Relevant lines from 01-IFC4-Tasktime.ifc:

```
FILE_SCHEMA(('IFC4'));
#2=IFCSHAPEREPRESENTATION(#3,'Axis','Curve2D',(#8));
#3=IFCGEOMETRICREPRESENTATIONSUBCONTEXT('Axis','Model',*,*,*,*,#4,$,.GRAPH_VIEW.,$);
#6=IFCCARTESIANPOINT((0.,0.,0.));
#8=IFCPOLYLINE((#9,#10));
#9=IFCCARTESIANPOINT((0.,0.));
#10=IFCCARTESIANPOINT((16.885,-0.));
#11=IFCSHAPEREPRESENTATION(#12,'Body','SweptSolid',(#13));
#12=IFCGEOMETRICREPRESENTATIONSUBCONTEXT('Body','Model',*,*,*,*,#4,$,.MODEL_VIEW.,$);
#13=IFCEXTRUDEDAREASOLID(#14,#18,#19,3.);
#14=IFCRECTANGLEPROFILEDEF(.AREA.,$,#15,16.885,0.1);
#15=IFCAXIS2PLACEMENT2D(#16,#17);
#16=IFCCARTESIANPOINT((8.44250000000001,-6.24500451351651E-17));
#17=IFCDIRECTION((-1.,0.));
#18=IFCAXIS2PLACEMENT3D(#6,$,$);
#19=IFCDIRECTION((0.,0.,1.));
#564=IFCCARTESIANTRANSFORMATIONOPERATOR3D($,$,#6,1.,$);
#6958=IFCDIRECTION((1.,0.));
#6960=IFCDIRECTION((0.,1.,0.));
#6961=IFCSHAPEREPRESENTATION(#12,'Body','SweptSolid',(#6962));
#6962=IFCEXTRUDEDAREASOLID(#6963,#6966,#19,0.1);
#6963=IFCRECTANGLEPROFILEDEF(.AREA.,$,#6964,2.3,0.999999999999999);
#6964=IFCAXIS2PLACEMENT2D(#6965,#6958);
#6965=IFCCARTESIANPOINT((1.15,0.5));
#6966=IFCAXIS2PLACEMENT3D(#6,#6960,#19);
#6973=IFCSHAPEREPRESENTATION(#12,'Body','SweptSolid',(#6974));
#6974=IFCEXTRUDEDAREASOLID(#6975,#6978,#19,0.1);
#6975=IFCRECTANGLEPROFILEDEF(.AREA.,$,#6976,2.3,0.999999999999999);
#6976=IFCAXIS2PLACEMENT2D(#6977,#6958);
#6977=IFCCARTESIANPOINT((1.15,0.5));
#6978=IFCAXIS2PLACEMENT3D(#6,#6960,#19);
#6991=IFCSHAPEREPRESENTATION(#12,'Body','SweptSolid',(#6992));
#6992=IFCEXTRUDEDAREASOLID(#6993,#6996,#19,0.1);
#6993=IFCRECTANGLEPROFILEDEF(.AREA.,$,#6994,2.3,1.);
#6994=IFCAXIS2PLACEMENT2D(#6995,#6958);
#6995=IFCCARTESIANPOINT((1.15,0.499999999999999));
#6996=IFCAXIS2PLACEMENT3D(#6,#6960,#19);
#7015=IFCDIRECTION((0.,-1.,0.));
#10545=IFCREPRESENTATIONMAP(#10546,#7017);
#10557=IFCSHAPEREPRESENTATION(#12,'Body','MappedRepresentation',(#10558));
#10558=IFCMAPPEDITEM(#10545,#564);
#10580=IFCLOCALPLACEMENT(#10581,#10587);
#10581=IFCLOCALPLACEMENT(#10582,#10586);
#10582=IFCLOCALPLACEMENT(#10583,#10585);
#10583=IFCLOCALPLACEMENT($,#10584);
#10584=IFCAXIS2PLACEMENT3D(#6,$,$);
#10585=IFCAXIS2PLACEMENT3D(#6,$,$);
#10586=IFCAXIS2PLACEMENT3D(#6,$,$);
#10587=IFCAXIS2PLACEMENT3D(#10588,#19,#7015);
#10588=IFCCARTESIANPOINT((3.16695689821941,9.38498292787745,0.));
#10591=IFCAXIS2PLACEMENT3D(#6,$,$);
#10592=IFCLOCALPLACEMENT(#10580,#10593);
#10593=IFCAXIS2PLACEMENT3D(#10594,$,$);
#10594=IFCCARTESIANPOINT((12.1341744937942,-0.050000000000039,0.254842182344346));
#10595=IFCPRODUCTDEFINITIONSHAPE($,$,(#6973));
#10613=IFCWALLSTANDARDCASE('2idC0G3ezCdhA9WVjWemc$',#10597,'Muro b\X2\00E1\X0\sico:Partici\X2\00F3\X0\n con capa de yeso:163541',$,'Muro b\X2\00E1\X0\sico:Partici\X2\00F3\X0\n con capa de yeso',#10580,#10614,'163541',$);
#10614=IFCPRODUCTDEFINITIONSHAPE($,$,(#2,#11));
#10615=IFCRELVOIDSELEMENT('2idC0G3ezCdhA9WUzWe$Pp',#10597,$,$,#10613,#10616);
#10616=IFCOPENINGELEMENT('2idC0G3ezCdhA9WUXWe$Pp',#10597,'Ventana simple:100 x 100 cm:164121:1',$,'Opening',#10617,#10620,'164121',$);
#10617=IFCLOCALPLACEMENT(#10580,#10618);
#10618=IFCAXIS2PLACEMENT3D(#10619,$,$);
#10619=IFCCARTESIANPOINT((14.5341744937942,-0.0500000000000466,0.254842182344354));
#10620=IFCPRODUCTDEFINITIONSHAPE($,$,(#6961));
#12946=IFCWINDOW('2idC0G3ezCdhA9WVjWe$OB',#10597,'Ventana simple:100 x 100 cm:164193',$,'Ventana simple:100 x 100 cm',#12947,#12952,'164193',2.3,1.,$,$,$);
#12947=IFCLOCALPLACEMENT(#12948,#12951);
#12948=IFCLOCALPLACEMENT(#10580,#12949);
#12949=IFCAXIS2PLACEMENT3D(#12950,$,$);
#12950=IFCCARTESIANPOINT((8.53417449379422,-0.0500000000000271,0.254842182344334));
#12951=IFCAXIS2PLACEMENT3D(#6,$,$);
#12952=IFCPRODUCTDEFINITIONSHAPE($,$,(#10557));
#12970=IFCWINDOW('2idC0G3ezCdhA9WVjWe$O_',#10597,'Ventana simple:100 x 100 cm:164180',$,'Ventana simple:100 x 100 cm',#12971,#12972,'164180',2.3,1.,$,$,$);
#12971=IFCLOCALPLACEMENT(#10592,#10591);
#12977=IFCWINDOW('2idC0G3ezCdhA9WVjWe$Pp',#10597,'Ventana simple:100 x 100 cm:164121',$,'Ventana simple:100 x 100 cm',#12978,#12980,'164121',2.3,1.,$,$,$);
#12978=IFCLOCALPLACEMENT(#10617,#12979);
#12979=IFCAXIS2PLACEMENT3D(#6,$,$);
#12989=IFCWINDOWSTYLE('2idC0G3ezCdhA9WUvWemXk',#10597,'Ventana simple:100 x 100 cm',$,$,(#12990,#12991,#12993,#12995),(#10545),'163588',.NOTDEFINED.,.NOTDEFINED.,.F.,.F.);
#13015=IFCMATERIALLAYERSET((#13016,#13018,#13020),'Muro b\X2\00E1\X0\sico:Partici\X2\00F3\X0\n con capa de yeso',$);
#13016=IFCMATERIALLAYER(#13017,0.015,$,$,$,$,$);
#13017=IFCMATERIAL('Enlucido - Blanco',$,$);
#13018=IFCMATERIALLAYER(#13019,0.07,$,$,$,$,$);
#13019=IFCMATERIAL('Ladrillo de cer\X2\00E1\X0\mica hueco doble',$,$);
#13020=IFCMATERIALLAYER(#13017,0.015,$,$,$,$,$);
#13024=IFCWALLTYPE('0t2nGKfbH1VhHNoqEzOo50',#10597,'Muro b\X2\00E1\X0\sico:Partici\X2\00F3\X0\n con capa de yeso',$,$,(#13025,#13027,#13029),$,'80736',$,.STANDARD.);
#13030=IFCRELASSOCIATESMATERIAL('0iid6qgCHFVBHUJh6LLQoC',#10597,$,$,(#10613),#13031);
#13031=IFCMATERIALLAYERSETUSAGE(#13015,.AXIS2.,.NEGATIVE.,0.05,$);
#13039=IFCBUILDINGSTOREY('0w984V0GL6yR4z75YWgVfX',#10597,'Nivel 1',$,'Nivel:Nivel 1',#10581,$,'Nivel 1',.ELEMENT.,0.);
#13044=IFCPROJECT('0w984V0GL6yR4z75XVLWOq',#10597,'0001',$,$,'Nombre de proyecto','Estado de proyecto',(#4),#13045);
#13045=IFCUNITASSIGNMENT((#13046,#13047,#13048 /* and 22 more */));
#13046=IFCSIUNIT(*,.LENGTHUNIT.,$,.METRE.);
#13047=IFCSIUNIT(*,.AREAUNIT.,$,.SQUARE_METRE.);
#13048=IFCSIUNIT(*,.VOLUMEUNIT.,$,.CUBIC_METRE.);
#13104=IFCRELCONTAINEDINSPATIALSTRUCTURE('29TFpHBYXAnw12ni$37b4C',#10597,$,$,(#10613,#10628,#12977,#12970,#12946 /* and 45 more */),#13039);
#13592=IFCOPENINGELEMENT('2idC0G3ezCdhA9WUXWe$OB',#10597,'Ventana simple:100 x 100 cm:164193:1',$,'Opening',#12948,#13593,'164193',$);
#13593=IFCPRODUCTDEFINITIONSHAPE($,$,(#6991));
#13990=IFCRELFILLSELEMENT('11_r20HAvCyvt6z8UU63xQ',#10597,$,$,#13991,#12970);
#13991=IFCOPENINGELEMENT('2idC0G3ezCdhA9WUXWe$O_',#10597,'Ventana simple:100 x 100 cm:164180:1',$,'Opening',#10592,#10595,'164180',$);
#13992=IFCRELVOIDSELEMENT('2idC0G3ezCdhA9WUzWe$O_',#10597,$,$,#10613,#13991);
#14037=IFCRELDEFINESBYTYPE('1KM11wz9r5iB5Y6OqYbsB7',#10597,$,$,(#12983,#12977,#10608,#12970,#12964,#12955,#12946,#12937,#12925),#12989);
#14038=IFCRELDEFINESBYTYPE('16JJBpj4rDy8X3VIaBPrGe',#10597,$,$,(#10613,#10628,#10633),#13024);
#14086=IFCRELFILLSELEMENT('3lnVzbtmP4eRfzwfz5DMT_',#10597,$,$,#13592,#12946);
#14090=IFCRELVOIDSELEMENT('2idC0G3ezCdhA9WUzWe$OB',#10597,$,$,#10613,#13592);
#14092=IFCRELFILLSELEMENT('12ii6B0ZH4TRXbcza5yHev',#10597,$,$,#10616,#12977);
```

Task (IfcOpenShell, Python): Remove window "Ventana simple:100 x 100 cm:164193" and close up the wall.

```python
import ifcopenshell
import ifcopenshell.api.feature
import ifcopenshell.api.root
import ifcopenshell.geom
import ifcopenshell.util.shape

model = ifcopenshell.open("01-IFC4-Tasktime.ifc")
settings = ifcopenshell.geom.settings()


def volume(element):
    """Net volume in cubic metres, openings subtracted."""
    shape = ifcopenshell.geom.create_shape(settings, element)
    return ifcopenshell.util.shape.get_volume(shape.geometry)


window = model.by_guid("2idC0G3ezCdhA9WVjWe$OB")
opening = window.FillsVoids[0].RelatingOpeningElement
wall = opening.VoidsElements[0].RelatingBuildingElement
before = volume(wall)

ifcopenshell.api.root.remove_product(model, product=window)
ifcopenshell.api.feature.remove_feature(model, feature=opening)

after = volume(wall)

print(f"wall volume {before:.3f} -> {after:.3f} m3")

model.write("01-IFC4-Tasktime-out.ifc")
```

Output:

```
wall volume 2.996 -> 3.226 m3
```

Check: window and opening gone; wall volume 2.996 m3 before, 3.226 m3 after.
